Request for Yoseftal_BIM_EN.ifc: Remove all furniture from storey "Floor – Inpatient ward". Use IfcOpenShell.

First a look at what the model holds.

```python
import ifcopenshell
import ifcopenshell.util.element

model = ifcopenshell.open("Yoseftal_BIM_EN.ifc")
print(model.schema)
storey = next(s for s in model.by_type("IfcBuildingStorey") if s.Name == "Floor – Inpatient ward")
furniture = [e for e in ifcopenshell.util.element.get_decomposition(storey) if e.is_a("IfcFurnishingElement")]
seen = {}
for e in furniture:
    element_type = ifcopenshell.util.element.get_type(e)
    name = element_type.Name if element_type not in (None, e) else None
    seen[name] = seen.get(name, 0) + 1
for name, count in sorted(seen.items(), key=str):
    print(count, "x", name)
```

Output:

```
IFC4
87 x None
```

```python
import ifcopenshell
import ifcopenshell.api.root
import ifcopenshell.util.element

model = ifcopenshell.open("Yoseftal_BIM_EN.ifc")

storey = next(s for s in model.by_type("IfcBuildingStorey") if s.Name == "Floor – Inpatient ward")
furniture = [e for e in ifcopenshell.util.element.get_decomposition(storey) if e.is_a("IfcFurnishingElement")]

for e in furniture:
    ifcopenshell.api.root.remove_product(model, product=e)
print(len(furniture), "removed")

model.write("Yoseftal_BIM_EN_rev.ifc")
```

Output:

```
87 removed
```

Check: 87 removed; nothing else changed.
